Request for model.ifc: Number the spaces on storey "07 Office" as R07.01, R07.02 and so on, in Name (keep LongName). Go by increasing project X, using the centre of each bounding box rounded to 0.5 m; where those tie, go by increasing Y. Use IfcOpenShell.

First a look at what the model holds.

```python
import ifcopenshell
import ifcopenshell.util.element
import ifcopenshell.util.placement

model = ifcopenshell.open("model.ifc")
print(model.schema)
storey = next(s for s in model.by_type("IfcBuildingStorey") if s.Name == "07 Office")
spaces = [e for e in ifcopenshell.util.element.get_decomposition(storey) if e.is_a("IfcSpace")]
for e in sorted(spaces, key=lambda e: e.id()):
    origin = ifcopenshell.util.placement.get_local_placement(e.ObjectPlacement)[:3, 3]
    print(e.id(), e.Name, e.LongName, origin.round(2) + 0.0, sep=" | ")
```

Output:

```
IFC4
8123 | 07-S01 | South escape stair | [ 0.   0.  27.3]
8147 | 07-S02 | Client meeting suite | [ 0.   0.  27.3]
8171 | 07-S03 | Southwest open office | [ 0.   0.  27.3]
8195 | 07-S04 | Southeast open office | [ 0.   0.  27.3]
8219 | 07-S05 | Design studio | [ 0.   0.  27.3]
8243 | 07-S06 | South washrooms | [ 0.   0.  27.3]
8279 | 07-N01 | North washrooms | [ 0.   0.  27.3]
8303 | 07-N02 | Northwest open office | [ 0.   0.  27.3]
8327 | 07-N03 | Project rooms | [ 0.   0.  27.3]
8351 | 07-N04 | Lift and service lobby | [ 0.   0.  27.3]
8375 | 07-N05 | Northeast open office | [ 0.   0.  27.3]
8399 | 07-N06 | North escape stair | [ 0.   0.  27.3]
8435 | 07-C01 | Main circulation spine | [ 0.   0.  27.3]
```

```python
import ifcopenshell
import ifcopenshell.geom
import ifcopenshell.util.element
import ifcopenshell.util.shape

model = ifcopenshell.open("model.ifc")
settings = ifcopenshell.geom.settings()
settings.set("use-world-coords", True)


def centre(element):
    shape = ifcopenshell.geom.create_shape(settings, element)
    return ifcopenshell.util.shape.get_bbox_centroid(shape.geometry)


storey = next(s for s in model.by_type("IfcBuildingStorey") if s.Name == "07 Office")
spaces = [e for e in ifcopenshell.util.element.get_decomposition(storey) if e.is_a("IfcSpace")]

# Insertion points can sit at a corner or the storey origin, so sort by the geometry (in metres).
centres = {e: centre(e) for e in spaces}
spaces.sort(key=lambda e: (round(centres[e][0] / 0.5), centres[e][1]))

for i, e in enumerate(spaces, start=1):
    number = f"R07.{i:02d}"
    e.Name = number
    print(e.id(), number)

model.write("model_edited.ifc")
```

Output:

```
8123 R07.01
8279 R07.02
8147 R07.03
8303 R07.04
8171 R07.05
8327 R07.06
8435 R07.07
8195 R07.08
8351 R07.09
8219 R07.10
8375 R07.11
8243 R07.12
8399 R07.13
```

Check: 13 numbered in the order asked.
